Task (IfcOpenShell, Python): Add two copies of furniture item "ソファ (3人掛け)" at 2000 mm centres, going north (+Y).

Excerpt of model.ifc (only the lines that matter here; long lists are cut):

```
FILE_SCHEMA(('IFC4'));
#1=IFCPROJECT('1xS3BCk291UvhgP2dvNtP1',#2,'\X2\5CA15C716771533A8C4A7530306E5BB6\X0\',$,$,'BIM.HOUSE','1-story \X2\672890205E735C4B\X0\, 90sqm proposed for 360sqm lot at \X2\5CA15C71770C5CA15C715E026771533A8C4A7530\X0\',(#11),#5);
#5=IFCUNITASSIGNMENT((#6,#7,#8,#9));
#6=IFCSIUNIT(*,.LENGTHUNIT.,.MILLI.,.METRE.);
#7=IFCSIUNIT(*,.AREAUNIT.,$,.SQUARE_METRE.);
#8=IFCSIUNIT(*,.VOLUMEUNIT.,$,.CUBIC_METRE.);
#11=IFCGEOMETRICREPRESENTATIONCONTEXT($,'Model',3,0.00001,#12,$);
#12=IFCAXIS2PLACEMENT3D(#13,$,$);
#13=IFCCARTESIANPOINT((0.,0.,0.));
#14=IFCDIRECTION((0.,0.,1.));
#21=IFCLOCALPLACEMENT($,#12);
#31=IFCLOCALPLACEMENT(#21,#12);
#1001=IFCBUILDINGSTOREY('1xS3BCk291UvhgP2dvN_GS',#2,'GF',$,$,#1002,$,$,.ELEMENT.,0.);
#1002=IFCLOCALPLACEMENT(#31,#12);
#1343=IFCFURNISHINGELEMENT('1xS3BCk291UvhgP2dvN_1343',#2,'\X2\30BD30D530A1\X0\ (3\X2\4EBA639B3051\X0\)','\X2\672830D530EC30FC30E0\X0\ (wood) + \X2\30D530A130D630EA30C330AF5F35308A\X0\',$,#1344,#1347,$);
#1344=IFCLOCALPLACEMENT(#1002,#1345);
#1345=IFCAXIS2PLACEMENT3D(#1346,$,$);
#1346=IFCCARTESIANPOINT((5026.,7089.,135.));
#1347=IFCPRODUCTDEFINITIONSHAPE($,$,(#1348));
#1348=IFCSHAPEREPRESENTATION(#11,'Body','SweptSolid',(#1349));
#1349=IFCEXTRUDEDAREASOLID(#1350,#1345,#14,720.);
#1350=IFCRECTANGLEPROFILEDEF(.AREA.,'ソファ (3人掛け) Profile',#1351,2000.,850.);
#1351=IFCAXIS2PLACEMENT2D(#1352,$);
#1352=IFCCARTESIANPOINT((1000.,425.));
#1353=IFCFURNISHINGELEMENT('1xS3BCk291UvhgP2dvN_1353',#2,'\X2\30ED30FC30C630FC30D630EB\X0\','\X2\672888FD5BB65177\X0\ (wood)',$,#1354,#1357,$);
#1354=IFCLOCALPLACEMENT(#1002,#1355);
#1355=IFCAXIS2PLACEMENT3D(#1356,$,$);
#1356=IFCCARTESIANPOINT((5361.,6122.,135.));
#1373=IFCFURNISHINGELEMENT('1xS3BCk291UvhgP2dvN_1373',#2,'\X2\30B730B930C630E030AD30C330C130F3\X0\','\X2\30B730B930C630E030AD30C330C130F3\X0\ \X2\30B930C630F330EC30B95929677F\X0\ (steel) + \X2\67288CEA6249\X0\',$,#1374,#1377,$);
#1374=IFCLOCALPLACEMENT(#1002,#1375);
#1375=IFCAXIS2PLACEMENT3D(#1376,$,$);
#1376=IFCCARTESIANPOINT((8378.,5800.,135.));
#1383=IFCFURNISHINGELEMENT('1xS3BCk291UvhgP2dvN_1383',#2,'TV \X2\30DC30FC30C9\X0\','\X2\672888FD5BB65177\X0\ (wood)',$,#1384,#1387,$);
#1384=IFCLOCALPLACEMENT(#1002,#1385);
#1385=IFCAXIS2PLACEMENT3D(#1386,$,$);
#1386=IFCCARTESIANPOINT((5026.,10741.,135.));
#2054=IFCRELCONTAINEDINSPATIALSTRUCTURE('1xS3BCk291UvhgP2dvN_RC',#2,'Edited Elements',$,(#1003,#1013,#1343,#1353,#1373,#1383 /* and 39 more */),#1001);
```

```python
import numpy as np
import ifcopenshell
import ifcopenshell.api.geometry
import ifcopenshell.api.root
import ifcopenshell.util.element
import ifcopenshell.util.placement
import ifcopenshell.util.unit

model = ifcopenshell.open("model.ifc")
unit_scale = ifcopenshell.util.unit.calculate_unit_scale(model)


def reuse_history(source, copy):
    """copy_class also copies each property set's owner history, people and application; keep the originals."""
    for rel in copy.IsDefinedBy:
        if rel.is_a("IfcRelDefinesByProperties") and (history := rel.RelatingPropertyDefinition.OwnerHistory):
            rel.RelatingPropertyDefinition.OwnerHistory = source.OwnerHistory
            ifcopenshell.util.element.remove_deep2(model, history)


source = model.by_guid("1xS3BCk291UvhgP2dvN_1343")
base = ifcopenshell.util.placement.get_local_placement(source.ObjectPlacement)
step = np.array([0.0, 1.0, 0.0]) * 2 / unit_scale

for i in range(1, 3):
    copy = ifcopenshell.api.root.copy_class(model, product=source)
    copy.Representation = ifcopenshell.util.element.copy_deep(
        model, source.Representation, exclude=["IfcGeometricRepresentationContext", "IfcRepresentationMap"]
    )
    reuse_history(source, copy)
    matrix = base.copy()
    matrix[:3, 3] += i * step
    print("added at", matrix[:3, 3].round(3) + 0.0)
    ifcopenshell.api.geometry.edit_object_placement(model, product=copy, matrix=matrix, is_si=False)

model.write("model_rev.ifc")
```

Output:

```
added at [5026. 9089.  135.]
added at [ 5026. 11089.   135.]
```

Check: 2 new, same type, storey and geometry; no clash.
